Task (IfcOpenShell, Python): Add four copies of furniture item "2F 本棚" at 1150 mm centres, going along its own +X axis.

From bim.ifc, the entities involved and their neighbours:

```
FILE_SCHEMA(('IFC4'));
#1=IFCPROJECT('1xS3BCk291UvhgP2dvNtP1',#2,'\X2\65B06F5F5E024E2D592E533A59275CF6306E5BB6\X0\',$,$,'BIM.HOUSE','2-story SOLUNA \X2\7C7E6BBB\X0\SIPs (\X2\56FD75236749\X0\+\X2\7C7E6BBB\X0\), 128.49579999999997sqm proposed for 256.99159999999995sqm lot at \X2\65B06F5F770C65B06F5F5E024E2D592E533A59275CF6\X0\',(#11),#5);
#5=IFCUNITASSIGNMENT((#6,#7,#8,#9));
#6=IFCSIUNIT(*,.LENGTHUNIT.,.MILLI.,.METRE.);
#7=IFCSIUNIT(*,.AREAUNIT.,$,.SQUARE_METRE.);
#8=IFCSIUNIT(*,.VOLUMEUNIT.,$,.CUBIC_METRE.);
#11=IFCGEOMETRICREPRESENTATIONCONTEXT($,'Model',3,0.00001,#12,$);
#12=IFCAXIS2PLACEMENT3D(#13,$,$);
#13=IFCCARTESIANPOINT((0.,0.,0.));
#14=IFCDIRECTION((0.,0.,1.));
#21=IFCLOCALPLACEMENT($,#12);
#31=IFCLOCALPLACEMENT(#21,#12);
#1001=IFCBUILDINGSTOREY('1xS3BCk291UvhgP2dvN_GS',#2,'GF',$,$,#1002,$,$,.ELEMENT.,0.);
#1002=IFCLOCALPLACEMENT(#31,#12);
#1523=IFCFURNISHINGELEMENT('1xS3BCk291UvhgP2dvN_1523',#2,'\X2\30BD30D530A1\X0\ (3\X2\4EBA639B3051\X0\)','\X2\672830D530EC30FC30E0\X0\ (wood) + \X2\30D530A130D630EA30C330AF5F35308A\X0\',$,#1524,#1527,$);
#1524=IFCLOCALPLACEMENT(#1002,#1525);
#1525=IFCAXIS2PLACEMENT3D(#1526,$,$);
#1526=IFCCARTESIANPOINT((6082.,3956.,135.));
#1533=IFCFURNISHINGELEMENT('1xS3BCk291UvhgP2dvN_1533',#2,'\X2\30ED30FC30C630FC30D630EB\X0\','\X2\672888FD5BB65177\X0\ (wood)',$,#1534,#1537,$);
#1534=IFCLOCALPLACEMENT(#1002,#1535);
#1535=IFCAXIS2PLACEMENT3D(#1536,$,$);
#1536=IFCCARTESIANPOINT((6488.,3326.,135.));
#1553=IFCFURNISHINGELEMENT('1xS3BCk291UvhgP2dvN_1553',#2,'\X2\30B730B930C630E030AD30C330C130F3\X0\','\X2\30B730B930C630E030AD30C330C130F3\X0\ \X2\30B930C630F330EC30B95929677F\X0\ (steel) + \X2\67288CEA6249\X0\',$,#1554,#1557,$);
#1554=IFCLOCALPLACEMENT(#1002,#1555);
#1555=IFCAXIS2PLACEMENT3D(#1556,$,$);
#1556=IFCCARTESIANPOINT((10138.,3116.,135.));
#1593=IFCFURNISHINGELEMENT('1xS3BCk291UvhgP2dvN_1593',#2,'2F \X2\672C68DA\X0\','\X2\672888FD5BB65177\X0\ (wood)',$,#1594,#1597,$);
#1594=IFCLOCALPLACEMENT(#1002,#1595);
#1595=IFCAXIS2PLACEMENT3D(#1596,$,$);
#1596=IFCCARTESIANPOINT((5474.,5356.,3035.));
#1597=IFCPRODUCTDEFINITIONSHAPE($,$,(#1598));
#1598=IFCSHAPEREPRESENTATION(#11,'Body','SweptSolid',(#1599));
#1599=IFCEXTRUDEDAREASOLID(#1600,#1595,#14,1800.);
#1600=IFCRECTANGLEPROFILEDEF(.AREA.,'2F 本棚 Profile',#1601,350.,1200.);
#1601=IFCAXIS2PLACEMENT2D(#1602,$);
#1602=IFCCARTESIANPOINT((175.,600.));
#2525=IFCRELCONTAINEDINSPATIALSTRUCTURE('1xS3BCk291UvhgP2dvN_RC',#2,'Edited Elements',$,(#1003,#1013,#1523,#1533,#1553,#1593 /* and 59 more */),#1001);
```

```python
import ifcopenshell
import ifcopenshell.api.geometry
import ifcopenshell.api.root
import ifcopenshell.util.element
import ifcopenshell.util.placement
import ifcopenshell.util.unit

model = ifcopenshell.open("bim.ifc")
unit_scale = ifcopenshell.util.unit.calculate_unit_scale(model)


def reuse_history(source, copy):
    """copy_class also copies each property set's owner history, people and application; keep the originals."""
    for rel in copy.IsDefinedBy:
        if rel.is_a("IfcRelDefinesByProperties") and (history := rel.RelatingPropertyDefinition.OwnerHistory):
            rel.RelatingPropertyDefinition.OwnerHistory = source.OwnerHistory
            ifcopenshell.util.element.remove_deep2(model, history)


source = model.by_guid("1xS3BCk291UvhgP2dvN_1593")
base = ifcopenshell.util.placement.get_local_placement(source.ObjectPlacement)
step = base[:3, 0] * 1.15 / unit_scale

for i in range(1, 5):
    copy = ifcopenshell.api.root.copy_class(model, product=source)
    copy.Representation = ifcopenshell.util.element.copy_deep(
        model, source.Representation, exclude=["IfcGeometricRepresentationContext", "IfcRepresentationMap"]
    )
    reuse_history(source, copy)
    matrix = base.copy()
    matrix[:3, 3] += i * step
    print("added at", matrix[:3, 3].round(3) + 0.0)
    ifcopenshell.api.geometry.edit_object_placement(model, product=copy, matrix=matrix, is_si=False)

model.write("bim-out.ifc")
```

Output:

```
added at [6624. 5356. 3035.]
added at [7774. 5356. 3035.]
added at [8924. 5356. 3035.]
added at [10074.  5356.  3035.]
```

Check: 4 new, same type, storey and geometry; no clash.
